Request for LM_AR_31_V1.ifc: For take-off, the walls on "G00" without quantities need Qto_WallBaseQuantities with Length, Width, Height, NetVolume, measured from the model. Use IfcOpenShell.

First a look at what the model holds.

```python
import ifcopenshell
import ifcopenshell.util.element
import ifcopenshell.util.unit

model = ifcopenshell.open("LM_AR_31_V1.ifc")
print(model.schema)
for unit_type in ("LENGTHUNIT", "AREAUNIT", "VOLUMEUNIT"):
    print(unit_type, ifcopenshell.util.unit.calculate_unit_scale(model, unit_type))
storey = next(s for s in model.by_type("IfcBuildingStorey") if s.Name == "G00")
walls = [e for e in ifcopenshell.util.element.get_decomposition(storey) if e.is_a("IfcWall")]
for e in sorted(walls, key=lambda e: e.id()):
    print(e.id(), e.is_a(), e.Name, list(ifcopenshell.util.element.get_psets(e, qtos_only=True)), sep=" | ")
```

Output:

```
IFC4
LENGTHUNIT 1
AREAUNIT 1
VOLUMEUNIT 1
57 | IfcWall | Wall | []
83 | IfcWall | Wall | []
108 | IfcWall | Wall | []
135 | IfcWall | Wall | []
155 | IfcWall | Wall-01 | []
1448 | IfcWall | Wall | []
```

```python
import ifcopenshell
import ifcopenshell.api.pset
import ifcopenshell.geom
import ifcopenshell.util.element
import ifcopenshell.util.shape
import ifcopenshell.util.unit

model = ifcopenshell.open("LM_AR_31_V1.ifc")
unit_scale = ifcopenshell.util.unit.calculate_unit_scale(model)
volume_scale = ifcopenshell.util.unit.calculate_unit_scale(model, "VOLUMEUNIT")
settings = ifcopenshell.geom.settings()

storey = next(s for s in model.by_type("IfcBuildingStorey") if s.Name == "G00")
walls = [e for e in ifcopenshell.util.element.get_decomposition(storey) if e.is_a("IfcWall")]

for e in sorted(walls, key=lambda e: e.id()):
    if ifcopenshell.util.element.get_psets(e, qtos_only=True, should_inherit=False):
        continue
    # Geometry comes back in metres, in the element's own axes.
    shape = ifcopenshell.geom.create_shape(settings, e)
    values = {
        "Length": ifcopenshell.util.shape.get_x(shape.geometry) / unit_scale,
        "Width": ifcopenshell.util.shape.get_y(shape.geometry) / unit_scale,
        "Height": ifcopenshell.util.shape.get_z(shape.geometry) / unit_scale,
        "NetVolume": ifcopenshell.util.shape.get_volume(shape.geometry) / volume_scale,
    }
    qto = ifcopenshell.api.pset.add_qto(model, product=e, name="Qto_WallBaseQuantities")
    ifcopenshell.api.pset.edit_qto(model, qto=qto, properties=values)
    print(e.id(), {k: round(v, 3) for k, v in values.items()})

model.write("LM_AR_31_V1_v2.ifc")
```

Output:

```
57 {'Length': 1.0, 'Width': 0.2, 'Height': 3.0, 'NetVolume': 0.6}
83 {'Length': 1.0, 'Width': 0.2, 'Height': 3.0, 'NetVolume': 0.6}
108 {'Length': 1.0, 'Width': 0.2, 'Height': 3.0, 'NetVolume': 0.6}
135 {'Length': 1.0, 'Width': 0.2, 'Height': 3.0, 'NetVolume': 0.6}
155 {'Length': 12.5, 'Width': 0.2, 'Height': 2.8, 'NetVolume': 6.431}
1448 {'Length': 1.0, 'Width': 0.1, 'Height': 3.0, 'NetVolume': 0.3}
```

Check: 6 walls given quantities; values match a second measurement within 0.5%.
